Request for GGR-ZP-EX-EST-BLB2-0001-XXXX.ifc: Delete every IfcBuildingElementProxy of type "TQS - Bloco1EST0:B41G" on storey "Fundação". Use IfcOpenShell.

First a look at what the model holds.

```python
import ifcopenshell
import ifcopenshell.util.element

model = ifcopenshell.open("GGR-ZP-EX-EST-BLB2-0001-XXXX.ifc")
print(model.schema)
storey = next(s for s in model.by_type("IfcBuildingStorey") if s.Name == "Fundação")
proxies = [e for e in ifcopenshell.util.element.get_decomposition(storey) if e.is_a("IfcBuildingElementProxy")]
seen = {}
for e in proxies:
    element_type = ifcopenshell.util.element.get_type(e)
    name = element_type.Name if element_type not in (None, e) else None
    seen[name] = seen.get(name, 0) + 1
for name, count in sorted(seen.items(), key=str):
    print(count, "x", name)
```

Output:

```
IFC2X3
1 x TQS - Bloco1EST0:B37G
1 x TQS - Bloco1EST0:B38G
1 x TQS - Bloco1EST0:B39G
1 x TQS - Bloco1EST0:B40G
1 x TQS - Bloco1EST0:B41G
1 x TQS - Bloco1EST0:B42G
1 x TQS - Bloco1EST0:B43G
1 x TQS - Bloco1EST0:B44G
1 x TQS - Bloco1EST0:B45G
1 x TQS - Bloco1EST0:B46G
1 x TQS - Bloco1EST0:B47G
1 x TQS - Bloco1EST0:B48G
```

```python
import ifcopenshell
import ifcopenshell.api.root
import ifcopenshell.util.element

model = ifcopenshell.open("GGR-ZP-EX-EST-BLB2-0001-XXXX.ifc")

storey = next(s for s in model.by_type("IfcBuildingStorey") if s.Name == "Fundação")
proxies = [e for e in ifcopenshell.util.element.get_decomposition(storey) if e.is_a("IfcBuildingElementProxy")]
targets = [e for e in proxies if (t := ifcopenshell.util.element.get_type(e)) not in (None, e) and t.Name == "TQS - Bloco1EST0:B41G"]

for e in targets:
    ifcopenshell.api.root.remove_product(model, product=e)
print(len(targets), "removed")

model.write("GGR-ZP-EX-EST-BLB2-0001-XXXX_v2.ifc")
```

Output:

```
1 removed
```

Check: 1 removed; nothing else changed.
